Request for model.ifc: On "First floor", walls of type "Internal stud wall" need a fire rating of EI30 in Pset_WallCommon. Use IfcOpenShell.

First a look at what the model holds.

```python
import ifcopenshell
import ifcopenshell.util.element

model = ifcopenshell.open("model.ifc")
print(model.schema)
storey = next(s for s in model.by_type("IfcBuildingStorey") if s.Name == "First floor")
walls = [e for e in ifcopenshell.util.element.get_decomposition(storey) if e.is_a("IfcWall")]
seen = {}
for e in walls:
    element_type = ifcopenshell.util.element.get_type(e)
    key = (element_type.Name if element_type != e and element_type else None, ifcopenshell.util.element.get_pset(e, "Pset_WallCommon", "FireRating"))
    seen[key] = seen.get(key, 0) + 1
for (name, value), count in sorted(seen.items(), key=str):
    print(count, "x", name, "|", value)
```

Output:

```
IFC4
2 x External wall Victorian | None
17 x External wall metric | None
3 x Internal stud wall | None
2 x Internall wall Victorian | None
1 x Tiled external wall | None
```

```python
import ifcopenshell
import ifcopenshell.api.pset
import ifcopenshell.util.element

model = ifcopenshell.open("model.ifc")

storey = next(s for s in model.by_type("IfcBuildingStorey") if s.Name == "First floor")
walls = [e for e in ifcopenshell.util.element.get_decomposition(storey) if e.is_a("IfcWall")]

count = 0
for e in walls:
    element_type = ifcopenshell.util.element.get_type(e)
    if element_type in (None, e) or element_type.Name != "Internal stud wall":
        continue
    # add_pset returns the element's existing set when there is one.
    pset = ifcopenshell.api.pset.add_pset(model, product=e, name="Pset_WallCommon")
    ifcopenshell.api.pset.edit_pset(model, pset=pset, properties={"FireRating": "EI30"})
    count += 1

print(count, "walls updated")

model.write("model_rev.ifc")
```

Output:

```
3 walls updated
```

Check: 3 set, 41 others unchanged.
